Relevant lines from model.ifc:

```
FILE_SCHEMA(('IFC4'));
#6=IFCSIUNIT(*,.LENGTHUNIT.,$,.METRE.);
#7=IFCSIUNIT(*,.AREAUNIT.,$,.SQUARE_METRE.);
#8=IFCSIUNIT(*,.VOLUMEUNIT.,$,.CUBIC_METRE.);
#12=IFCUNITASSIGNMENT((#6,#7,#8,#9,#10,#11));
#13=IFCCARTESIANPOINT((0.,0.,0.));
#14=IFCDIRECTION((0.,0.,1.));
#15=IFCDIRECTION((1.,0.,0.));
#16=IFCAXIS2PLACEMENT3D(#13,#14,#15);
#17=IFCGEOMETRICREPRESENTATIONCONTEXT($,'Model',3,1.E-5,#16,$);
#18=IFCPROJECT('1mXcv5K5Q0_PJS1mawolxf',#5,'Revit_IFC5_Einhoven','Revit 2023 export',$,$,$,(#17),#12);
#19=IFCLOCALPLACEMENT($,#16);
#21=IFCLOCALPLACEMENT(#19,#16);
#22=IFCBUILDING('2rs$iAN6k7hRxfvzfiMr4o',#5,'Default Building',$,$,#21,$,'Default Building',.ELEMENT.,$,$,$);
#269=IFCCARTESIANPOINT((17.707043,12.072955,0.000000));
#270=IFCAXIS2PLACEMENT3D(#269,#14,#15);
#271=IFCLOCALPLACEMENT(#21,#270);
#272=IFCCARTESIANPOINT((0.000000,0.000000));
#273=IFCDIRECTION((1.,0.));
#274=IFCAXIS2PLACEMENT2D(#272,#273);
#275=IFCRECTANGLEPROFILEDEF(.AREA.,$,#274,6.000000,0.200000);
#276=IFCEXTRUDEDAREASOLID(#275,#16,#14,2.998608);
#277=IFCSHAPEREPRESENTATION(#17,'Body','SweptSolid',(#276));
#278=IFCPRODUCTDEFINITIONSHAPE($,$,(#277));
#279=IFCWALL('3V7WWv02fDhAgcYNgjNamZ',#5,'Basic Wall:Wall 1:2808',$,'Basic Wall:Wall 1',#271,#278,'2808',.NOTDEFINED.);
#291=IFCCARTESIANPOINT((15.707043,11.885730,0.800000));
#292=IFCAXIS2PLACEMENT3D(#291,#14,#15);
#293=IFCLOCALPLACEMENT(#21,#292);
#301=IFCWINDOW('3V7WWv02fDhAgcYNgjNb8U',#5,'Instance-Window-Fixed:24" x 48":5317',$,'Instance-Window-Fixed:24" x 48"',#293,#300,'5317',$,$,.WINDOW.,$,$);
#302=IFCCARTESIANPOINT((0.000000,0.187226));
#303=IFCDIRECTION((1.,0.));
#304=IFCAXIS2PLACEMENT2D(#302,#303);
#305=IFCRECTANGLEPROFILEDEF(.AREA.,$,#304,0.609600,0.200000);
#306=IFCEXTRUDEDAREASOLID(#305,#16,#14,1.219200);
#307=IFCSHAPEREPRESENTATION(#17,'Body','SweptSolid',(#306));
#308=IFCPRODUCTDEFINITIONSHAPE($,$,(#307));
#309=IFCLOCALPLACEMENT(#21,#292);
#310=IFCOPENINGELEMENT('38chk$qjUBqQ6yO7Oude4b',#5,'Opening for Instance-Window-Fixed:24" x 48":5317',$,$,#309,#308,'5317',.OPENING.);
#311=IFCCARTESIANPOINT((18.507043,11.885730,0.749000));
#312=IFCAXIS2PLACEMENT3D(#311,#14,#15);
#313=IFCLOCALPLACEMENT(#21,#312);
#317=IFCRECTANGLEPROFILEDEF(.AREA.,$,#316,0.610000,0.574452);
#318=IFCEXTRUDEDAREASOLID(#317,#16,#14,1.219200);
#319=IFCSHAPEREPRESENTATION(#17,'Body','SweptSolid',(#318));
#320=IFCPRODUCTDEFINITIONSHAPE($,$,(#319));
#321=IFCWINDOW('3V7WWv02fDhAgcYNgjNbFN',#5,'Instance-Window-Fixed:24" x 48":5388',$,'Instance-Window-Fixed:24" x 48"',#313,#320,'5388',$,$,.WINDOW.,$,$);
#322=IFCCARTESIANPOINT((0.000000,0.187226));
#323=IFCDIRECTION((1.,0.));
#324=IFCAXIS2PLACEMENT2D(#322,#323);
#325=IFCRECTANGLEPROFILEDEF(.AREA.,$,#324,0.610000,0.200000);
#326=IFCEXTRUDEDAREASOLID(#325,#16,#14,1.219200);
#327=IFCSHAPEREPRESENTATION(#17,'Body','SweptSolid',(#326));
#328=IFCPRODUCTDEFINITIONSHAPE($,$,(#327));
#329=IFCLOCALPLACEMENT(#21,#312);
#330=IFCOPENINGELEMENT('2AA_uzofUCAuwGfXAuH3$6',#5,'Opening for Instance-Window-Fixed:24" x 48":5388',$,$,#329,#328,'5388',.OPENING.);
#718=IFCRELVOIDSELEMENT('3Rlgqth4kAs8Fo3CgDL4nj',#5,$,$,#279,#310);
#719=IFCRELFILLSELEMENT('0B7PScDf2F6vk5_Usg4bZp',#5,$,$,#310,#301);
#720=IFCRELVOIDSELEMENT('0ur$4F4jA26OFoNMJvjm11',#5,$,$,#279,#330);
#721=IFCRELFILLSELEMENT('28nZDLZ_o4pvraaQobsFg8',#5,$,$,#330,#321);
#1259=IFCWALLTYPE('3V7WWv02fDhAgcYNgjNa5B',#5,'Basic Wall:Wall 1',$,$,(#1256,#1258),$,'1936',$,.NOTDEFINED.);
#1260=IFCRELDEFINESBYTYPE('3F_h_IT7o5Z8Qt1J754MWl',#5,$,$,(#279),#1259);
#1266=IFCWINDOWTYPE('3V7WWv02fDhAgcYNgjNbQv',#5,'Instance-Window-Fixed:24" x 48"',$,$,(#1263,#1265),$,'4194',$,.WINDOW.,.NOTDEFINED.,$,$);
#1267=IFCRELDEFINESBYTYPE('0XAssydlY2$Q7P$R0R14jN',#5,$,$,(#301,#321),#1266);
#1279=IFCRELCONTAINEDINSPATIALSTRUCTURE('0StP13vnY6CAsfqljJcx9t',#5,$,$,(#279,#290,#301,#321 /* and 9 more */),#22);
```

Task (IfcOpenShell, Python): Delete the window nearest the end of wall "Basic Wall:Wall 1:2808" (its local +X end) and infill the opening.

```python
import ifcopenshell
import ifcopenshell.api.feature
import ifcopenshell.api.root
import ifcopenshell.geom
import ifcopenshell.util.shape

model = ifcopenshell.open("model.ifc")
settings = ifcopenshell.geom.settings()


def volume(element):
    """Net volume in cubic metres, openings subtracted."""
    shape = ifcopenshell.geom.create_shape(settings, element)
    return ifcopenshell.util.shape.get_volume(shape.geometry)


window = model.by_guid("3V7WWv02fDhAgcYNgjNbFN")
opening = window.FillsVoids[0].RelatingOpeningElement
wall = opening.VoidsElements[0].RelatingBuildingElement
before = volume(wall)

ifcopenshell.api.root.remove_product(model, product=window)
ifcopenshell.api.feature.remove_feature(model, feature=opening)

after = volume(wall)

print(f"wall volume {before:.3f} -> {after:.3f} m3")

model.write("model_updated.ifc")
```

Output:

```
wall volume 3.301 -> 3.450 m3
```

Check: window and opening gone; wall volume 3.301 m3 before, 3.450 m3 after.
